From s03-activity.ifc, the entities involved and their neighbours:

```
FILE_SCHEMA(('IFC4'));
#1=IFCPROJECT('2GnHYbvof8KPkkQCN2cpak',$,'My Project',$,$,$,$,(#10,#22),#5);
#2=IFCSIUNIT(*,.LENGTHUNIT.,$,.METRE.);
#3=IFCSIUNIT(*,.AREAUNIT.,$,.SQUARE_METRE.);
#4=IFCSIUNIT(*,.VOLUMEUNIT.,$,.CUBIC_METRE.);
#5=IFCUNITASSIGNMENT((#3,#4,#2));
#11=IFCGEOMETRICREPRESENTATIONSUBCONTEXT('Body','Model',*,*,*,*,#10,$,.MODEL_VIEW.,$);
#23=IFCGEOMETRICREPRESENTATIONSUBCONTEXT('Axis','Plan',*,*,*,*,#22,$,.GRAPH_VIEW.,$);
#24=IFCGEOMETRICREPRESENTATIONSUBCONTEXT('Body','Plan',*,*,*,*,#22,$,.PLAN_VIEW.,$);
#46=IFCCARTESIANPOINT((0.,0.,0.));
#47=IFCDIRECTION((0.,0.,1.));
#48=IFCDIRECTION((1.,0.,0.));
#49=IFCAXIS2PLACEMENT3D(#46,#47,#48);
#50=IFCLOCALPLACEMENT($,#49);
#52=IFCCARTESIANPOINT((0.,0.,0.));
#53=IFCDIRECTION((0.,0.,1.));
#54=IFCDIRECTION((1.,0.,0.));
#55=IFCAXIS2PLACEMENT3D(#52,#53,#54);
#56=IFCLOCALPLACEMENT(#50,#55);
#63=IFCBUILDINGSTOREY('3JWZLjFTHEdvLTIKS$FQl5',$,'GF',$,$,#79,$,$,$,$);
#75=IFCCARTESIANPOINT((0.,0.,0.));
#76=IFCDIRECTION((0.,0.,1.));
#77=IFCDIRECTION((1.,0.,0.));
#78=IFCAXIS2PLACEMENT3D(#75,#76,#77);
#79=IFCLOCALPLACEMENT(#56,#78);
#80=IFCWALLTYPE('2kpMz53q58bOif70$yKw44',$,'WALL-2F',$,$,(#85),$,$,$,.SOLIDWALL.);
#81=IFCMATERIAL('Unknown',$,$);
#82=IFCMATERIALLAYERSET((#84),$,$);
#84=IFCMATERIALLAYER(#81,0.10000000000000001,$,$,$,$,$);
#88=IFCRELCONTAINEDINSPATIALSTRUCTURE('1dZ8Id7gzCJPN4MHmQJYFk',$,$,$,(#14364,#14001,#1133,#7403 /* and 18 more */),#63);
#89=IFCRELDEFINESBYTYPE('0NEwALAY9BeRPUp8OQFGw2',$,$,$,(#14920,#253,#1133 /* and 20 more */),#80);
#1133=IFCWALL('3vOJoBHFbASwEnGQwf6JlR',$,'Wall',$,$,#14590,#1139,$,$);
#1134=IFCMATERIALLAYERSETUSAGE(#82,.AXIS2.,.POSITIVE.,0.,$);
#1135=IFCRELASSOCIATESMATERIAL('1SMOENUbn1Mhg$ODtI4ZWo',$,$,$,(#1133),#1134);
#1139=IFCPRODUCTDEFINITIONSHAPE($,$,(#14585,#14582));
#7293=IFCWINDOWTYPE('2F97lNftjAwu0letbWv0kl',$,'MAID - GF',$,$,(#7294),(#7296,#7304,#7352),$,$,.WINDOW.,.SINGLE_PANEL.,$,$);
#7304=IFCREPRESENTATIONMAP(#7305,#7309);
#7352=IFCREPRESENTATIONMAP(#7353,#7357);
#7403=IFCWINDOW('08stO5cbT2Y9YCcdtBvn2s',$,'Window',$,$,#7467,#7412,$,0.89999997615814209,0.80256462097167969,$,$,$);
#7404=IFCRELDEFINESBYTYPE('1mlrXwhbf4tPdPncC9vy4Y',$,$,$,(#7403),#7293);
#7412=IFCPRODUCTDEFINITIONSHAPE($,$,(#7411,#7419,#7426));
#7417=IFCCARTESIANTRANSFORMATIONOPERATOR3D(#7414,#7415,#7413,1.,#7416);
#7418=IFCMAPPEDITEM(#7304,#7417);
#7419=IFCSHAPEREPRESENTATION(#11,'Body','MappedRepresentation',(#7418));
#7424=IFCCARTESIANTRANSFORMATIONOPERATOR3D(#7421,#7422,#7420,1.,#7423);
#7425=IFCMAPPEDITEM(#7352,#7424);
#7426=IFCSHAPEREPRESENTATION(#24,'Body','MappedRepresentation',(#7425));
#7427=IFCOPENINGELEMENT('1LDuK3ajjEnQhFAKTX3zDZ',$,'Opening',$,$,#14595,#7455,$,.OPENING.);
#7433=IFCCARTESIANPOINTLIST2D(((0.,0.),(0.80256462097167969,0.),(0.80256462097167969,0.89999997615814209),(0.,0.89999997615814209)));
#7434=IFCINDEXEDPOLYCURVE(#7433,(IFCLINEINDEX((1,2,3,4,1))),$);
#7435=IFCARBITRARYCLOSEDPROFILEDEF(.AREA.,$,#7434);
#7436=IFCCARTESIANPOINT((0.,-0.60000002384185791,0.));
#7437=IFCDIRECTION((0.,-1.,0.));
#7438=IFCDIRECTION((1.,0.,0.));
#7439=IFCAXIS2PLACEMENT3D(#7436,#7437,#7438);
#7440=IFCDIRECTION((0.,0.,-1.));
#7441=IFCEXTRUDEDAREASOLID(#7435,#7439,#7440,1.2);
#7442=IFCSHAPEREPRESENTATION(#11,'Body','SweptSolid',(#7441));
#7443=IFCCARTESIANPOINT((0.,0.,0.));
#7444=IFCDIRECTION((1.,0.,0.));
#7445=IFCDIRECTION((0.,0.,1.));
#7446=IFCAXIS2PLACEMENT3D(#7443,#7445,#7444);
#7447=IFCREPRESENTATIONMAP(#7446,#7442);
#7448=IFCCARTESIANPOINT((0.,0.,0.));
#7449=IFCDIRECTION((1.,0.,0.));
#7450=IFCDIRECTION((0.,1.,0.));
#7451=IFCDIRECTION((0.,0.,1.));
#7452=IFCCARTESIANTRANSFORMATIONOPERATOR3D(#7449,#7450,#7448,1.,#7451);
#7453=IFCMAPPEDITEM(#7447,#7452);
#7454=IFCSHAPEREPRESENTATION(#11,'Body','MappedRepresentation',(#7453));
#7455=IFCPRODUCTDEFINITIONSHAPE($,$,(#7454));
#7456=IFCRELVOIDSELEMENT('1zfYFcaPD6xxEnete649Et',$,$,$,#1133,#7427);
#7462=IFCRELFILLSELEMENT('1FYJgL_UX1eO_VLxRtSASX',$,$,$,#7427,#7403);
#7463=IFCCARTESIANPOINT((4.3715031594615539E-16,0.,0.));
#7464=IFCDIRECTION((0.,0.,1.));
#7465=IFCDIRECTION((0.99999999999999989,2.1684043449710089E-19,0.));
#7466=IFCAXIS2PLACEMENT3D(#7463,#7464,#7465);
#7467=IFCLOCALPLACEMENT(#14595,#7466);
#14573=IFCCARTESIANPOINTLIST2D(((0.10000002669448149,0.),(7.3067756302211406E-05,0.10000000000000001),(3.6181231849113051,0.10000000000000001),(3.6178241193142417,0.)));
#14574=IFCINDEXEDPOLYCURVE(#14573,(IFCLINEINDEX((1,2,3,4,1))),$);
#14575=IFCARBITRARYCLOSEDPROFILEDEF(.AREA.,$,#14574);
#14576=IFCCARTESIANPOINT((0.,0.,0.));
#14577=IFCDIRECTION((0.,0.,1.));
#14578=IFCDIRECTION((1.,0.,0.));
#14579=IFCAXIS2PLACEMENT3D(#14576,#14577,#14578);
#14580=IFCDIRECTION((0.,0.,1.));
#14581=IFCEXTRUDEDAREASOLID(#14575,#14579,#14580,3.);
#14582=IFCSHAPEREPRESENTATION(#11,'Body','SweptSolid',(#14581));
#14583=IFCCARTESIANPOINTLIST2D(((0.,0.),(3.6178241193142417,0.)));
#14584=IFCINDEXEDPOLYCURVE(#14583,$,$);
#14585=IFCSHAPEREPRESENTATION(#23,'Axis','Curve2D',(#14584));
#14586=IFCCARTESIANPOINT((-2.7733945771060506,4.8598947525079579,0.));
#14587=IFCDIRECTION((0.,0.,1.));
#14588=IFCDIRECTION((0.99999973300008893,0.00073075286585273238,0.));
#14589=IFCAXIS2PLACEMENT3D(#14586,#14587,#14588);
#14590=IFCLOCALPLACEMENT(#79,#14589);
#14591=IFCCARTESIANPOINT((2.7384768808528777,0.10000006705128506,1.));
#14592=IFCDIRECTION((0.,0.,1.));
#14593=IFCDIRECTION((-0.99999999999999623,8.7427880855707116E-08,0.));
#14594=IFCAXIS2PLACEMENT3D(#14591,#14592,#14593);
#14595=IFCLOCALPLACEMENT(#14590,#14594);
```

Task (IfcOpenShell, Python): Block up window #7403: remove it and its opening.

```python
import ifcopenshell
import ifcopenshell.api.feature
import ifcopenshell.api.root
import ifcopenshell.geom
import ifcopenshell.util.shape

model = ifcopenshell.open("s03-activity.ifc")
settings = ifcopenshell.geom.settings()


def volume(element):
    """Net volume in cubic metres, openings subtracted."""
    shape = ifcopenshell.geom.create_shape(settings, element)
    return ifcopenshell.util.shape.get_volume(shape.geometry)


window = model.by_id(7403)
opening = window.FillsVoids[0].RelatingOpeningElement
wall = opening.VoidsElements[0].RelatingBuildingElement
before = volume(wall)

ifcopenshell.api.root.remove_product(model, product=window)
ifcopenshell.api.feature.remove_feature(model, feature=opening)

after = volume(wall)

print(f"wall volume {before:.3f} -> {after:.3f} m3")

model.write("s03-activity_rev.ifc")
```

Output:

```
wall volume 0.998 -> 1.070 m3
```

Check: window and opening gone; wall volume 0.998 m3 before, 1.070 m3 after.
